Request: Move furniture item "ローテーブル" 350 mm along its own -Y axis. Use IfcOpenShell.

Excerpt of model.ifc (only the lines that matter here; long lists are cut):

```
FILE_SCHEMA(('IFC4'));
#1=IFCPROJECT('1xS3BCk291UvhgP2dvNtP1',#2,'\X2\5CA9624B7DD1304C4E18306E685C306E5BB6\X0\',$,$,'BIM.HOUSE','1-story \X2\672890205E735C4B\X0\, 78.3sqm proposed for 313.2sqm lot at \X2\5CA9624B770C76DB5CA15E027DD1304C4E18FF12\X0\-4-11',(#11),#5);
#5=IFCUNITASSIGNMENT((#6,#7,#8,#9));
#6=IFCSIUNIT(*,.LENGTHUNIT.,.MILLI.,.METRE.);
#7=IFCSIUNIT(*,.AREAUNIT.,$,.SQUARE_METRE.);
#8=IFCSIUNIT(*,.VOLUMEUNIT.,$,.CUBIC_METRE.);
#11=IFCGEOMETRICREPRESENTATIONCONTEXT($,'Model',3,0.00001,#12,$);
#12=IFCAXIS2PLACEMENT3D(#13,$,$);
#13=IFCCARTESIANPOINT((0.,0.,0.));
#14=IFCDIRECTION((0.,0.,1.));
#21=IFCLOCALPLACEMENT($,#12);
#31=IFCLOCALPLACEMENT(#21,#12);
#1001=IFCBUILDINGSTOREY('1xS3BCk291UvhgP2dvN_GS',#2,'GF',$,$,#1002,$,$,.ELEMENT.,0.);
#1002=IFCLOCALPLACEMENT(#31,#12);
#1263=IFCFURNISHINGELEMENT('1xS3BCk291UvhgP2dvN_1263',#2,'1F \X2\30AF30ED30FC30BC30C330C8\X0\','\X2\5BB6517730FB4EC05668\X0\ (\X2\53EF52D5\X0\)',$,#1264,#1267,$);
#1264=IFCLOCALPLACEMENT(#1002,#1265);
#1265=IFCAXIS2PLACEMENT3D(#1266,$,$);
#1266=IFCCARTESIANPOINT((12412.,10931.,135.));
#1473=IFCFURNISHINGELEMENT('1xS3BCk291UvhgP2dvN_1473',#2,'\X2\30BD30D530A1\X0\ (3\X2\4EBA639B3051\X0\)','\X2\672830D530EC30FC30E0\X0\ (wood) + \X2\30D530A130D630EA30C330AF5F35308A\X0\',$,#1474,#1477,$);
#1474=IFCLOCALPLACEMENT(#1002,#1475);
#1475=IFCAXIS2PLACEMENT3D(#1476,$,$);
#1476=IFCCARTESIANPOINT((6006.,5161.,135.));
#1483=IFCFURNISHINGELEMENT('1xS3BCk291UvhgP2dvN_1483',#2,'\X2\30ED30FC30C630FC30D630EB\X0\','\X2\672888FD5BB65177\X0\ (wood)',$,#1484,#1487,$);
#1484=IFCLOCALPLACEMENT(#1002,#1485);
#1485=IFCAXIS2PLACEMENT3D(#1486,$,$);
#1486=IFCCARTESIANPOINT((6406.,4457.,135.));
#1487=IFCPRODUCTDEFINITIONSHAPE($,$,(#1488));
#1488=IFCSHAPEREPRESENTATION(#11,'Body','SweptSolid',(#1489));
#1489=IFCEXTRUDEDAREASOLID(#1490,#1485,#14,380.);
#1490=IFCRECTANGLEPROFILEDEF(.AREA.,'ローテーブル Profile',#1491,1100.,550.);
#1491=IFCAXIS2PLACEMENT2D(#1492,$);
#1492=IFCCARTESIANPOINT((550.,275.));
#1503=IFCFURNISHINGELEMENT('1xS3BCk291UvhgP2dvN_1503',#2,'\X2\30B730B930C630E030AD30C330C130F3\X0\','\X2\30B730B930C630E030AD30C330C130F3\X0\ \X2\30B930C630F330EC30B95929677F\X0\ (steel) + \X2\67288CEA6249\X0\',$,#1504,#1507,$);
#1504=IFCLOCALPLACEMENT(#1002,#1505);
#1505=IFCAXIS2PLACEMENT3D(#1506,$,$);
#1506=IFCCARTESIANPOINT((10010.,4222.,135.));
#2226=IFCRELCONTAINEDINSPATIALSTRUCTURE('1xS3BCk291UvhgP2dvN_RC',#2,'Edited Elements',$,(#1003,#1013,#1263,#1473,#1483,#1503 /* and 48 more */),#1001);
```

```python
import ifcopenshell
import ifcopenshell.api.geometry
import ifcopenshell.util.placement
import ifcopenshell.util.unit

model = ifcopenshell.open("model.ifc")
unit_scale = ifcopenshell.util.unit.calculate_unit_scale(model)

item = model.by_id(1483)
matrix = ifcopenshell.util.placement.get_local_placement(item.ObjectPlacement)
matrix[:3, 3] -= matrix[:3, 1] * 0.35 / unit_scale
ifcopenshell.api.geometry.edit_object_placement(model, product=item, matrix=matrix, is_si=False)

print(ifcopenshell.util.placement.get_local_placement(item.ObjectPlacement).round(3) + 0.0)

model.write("model_edited.ifc")
```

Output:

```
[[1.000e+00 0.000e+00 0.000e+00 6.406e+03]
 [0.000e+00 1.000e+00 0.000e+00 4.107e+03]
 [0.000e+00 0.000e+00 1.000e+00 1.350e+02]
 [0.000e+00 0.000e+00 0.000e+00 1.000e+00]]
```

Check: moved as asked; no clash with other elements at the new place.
